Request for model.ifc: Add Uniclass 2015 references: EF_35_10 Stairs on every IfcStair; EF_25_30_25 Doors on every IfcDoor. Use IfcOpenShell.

First a look at what the model holds.

```python
import ifcopenshell

model = ifcopenshell.open("model.ifc")
print(model.schema)
print("classifications:", [c.Name for c in model.by_type("IfcClassification")])
for ifc_class in ("IfcDoor", "IfcRoof", "IfcStair", "IfcWall", "IfcWindow"):
    print(ifc_class, len(model.by_type(ifc_class)))
```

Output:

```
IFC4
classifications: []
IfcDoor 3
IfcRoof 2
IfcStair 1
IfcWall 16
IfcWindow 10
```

```python
import ifcopenshell
import ifcopenshell.api.classification

model = ifcopenshell.open("model.ifc")

system = ifcopenshell.api.classification.add_classification(model, classification="Uniclass 2015")

codes = {
    "IfcStair": ("EF_35_10", "Stairs"),
    "IfcDoor": ("EF_25_30_25", "Doors"),
}
for ifc_class, (code, name) in codes.items():
    products = model.by_type(ifc_class)
    ifcopenshell.api.classification.add_reference(
        model, products=products, classification=system, identification=code, name=name
    )
    print(code, len(products))

model.write("model-out.ifc")
```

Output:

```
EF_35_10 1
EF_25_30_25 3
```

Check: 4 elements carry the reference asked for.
